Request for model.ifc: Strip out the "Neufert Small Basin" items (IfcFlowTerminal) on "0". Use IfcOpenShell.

First a look at what the model holds.

```python
import ifcopenshell
import ifcopenshell.util.element

model = ifcopenshell.open("model.ifc")
print(model.schema)
storey = next(s for s in model.by_type("IfcBuildingStorey") if s.Name == "0")
terminals = [e for e in ifcopenshell.util.element.get_decomposition(storey) if e.is_a("IfcFlowTerminal")]
seen = {}
for e in terminals:
    element_type = ifcopenshell.util.element.get_type(e)
    name = element_type.Name if element_type not in (None, e) else None
    seen[name] = seen.get(name, 0) + 1
for name, count in sorted(seen.items(), key=str):
    print(count, "x", name)
```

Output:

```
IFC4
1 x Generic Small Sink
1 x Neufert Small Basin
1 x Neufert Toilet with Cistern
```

```python
import ifcopenshell
import ifcopenshell.api.root
import ifcopenshell.util.element

model = ifcopenshell.open("model.ifc")

storey = next(s for s in model.by_type("IfcBuildingStorey") if s.Name == "0")
terminals = [e for e in ifcopenshell.util.element.get_decomposition(storey) if e.is_a("IfcFlowTerminal")]
targets = [e for e in terminals if (t := ifcopenshell.util.element.get_type(e)) not in (None, e) and t.Name == "Neufert Small Basin"]

for e in targets:
    ifcopenshell.api.root.remove_product(model, product=e)
print(len(targets), "removed")

model.write("model_updated.ifc")
```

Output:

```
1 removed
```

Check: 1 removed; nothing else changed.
